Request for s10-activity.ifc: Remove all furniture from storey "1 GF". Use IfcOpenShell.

First a look at what the model holds.

```python
import ifcopenshell
import ifcopenshell.util.element

model = ifcopenshell.open("s10-activity.ifc")
print(model.schema)
storey = next(s for s in model.by_type("IfcBuildingStorey") if s.Name == "1 GF")
furniture = [e for e in ifcopenshell.util.element.get_decomposition(storey) if e.is_a("IfcFurnishingElement")]
seen = {}
for e in furniture:
    element_type = ifcopenshell.util.element.get_type(e)
    name = element_type.Name if element_type not in (None, e) else None
    seen[name] = seen.get(name, 0) + 1
for name, count in sorted(seen.items(), key=str):
    print(count, "x", name)
```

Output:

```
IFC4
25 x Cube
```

```python
import ifcopenshell
import ifcopenshell.api.root
import ifcopenshell.util.element

model = ifcopenshell.open("s10-activity.ifc")

storey = next(s for s in model.by_type("IfcBuildingStorey") if s.Name == "1 GF")
furniture = [e for e in ifcopenshell.util.element.get_decomposition(storey) if e.is_a("IfcFurnishingElement")]

for e in furniture:
    ifcopenshell.api.root.remove_product(model, product=e)
print(len(furniture), "removed")

model.write("s10-activity_edited.ifc")
```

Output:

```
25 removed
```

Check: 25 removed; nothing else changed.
